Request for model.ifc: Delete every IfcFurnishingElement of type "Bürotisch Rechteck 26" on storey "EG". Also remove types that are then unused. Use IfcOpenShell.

First a look at what the model holds.

```python
import ifcopenshell
import ifcopenshell.util.element

model = ifcopenshell.open("model.ifc")
print(model.schema)
storey = next(s for s in model.by_type("IfcBuildingStorey") if s.Name == "EG")
furniture = [e for e in ifcopenshell.util.element.get_decomposition(storey) if e.is_a("IfcFurnishingElement")]
seen = {}
for e in furniture:
    element_type = ifcopenshell.util.element.get_type(e)
    name = element_type.Name if element_type not in (None, e) else None
    seen[name] = seen.get(name, 0) + 1
for name, count in sorted(seen.items(), key=str):
    print(count, "x", name)
```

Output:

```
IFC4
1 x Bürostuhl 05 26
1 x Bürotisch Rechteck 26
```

```python
import ifcopenshell
import ifcopenshell.api.root
import ifcopenshell.util.element

model = ifcopenshell.open("model.ifc")

storey = next(s for s in model.by_type("IfcBuildingStorey") if s.Name == "EG")
furniture = [e for e in ifcopenshell.util.element.get_decomposition(storey) if e.is_a("IfcFurnishingElement")]
targets = [e for e in furniture if (t := ifcopenshell.util.element.get_type(e)) not in (None, e) and t.Name == "Bürotisch Rechteck 26"]
types = {ifcopenshell.util.element.get_type(e) for e in targets} - {None, *targets}

for e in targets:
    ifcopenshell.api.root.remove_product(model, product=e)
print(len(targets), "removed")

unused = [t for t in types if not ifcopenshell.util.element.get_types(t)]
for t in unused:
    ifcopenshell.api.root.remove_product(model, product=t)
print(len(unused), "unused types removed")

model.write("model-out.ifc")
```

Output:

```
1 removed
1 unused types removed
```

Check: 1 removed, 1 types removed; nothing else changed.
